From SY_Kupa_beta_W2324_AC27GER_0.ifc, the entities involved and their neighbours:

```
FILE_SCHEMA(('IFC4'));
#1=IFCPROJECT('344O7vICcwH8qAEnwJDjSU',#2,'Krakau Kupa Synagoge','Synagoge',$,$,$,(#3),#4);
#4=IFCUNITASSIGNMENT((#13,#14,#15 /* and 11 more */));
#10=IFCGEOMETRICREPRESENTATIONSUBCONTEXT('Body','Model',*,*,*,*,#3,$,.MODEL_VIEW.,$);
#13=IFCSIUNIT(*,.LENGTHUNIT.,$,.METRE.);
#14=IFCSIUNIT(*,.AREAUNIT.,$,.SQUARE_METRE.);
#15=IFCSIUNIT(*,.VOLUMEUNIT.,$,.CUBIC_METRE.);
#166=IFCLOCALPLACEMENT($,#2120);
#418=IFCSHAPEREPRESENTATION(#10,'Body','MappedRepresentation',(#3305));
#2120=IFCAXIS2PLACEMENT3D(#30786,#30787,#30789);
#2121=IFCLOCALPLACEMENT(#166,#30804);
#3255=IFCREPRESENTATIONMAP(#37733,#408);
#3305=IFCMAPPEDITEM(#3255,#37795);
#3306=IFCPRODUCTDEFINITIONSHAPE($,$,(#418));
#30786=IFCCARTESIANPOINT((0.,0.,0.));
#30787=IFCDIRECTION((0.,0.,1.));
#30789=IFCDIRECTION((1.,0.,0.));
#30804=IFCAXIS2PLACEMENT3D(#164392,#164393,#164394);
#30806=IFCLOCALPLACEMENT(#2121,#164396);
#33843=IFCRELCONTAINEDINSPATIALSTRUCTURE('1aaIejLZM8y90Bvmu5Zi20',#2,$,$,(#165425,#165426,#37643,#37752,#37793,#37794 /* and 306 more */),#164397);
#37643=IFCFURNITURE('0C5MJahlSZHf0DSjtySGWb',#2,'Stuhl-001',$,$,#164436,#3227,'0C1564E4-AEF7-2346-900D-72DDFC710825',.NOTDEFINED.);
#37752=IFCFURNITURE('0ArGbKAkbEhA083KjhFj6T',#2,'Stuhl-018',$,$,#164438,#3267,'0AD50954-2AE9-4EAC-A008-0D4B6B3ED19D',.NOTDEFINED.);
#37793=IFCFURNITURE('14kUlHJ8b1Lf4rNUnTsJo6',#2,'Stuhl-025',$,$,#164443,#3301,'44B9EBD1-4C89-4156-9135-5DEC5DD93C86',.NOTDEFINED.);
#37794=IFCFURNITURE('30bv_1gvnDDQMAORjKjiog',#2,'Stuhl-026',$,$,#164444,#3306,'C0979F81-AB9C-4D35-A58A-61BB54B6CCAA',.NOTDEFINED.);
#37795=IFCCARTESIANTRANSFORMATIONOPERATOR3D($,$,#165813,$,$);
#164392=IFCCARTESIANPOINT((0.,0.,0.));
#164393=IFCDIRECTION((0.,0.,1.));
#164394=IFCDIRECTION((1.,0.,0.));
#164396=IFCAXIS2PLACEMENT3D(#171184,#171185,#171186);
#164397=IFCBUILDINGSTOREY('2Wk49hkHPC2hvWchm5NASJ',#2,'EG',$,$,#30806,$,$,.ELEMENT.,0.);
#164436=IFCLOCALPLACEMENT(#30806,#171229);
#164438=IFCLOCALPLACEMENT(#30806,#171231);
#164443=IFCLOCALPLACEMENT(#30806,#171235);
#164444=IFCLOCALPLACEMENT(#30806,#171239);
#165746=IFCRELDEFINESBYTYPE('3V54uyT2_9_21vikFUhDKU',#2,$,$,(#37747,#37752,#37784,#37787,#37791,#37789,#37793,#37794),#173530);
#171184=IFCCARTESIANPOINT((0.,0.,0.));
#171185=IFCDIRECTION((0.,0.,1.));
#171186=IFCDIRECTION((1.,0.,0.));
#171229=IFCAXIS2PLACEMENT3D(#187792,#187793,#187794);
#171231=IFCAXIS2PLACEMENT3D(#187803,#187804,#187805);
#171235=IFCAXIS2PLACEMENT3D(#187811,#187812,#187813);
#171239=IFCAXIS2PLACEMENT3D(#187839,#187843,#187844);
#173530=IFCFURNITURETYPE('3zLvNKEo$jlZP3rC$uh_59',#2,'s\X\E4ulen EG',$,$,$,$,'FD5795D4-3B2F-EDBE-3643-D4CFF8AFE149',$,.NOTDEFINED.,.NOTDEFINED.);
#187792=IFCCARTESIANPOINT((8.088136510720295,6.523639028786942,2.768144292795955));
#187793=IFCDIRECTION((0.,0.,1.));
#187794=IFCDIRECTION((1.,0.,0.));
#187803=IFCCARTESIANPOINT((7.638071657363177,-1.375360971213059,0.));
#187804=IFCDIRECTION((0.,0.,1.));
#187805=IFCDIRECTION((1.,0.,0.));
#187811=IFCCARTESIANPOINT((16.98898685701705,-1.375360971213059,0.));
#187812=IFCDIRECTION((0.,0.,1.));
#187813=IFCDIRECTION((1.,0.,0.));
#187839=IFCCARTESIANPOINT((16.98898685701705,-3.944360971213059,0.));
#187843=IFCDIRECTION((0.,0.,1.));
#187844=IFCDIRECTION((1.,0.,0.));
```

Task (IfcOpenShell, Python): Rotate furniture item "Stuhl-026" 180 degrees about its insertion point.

```python
import ifcopenshell
import ifcopenshell.api.geometry
import ifcopenshell.util.placement

model = ifcopenshell.open("SY_Kupa_beta_W2324_AC27GER_0.ifc")

item = model.by_id(37794)
matrix = ifcopenshell.util.placement.get_local_placement(item.ObjectPlacement)
matrix = matrix @ ifcopenshell.util.placement.rotation(180, "Z")
ifcopenshell.api.geometry.edit_object_placement(model, product=item, matrix=matrix, is_si=False)

print(ifcopenshell.util.placement.get_local_placement(item.ObjectPlacement).round(3) + 0.0)

model.write("SY_Kupa_beta_W2324_AC27GER_0_rev.ifc")
```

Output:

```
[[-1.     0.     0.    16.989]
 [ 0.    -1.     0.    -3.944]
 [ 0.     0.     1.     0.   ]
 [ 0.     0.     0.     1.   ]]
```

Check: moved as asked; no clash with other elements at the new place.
